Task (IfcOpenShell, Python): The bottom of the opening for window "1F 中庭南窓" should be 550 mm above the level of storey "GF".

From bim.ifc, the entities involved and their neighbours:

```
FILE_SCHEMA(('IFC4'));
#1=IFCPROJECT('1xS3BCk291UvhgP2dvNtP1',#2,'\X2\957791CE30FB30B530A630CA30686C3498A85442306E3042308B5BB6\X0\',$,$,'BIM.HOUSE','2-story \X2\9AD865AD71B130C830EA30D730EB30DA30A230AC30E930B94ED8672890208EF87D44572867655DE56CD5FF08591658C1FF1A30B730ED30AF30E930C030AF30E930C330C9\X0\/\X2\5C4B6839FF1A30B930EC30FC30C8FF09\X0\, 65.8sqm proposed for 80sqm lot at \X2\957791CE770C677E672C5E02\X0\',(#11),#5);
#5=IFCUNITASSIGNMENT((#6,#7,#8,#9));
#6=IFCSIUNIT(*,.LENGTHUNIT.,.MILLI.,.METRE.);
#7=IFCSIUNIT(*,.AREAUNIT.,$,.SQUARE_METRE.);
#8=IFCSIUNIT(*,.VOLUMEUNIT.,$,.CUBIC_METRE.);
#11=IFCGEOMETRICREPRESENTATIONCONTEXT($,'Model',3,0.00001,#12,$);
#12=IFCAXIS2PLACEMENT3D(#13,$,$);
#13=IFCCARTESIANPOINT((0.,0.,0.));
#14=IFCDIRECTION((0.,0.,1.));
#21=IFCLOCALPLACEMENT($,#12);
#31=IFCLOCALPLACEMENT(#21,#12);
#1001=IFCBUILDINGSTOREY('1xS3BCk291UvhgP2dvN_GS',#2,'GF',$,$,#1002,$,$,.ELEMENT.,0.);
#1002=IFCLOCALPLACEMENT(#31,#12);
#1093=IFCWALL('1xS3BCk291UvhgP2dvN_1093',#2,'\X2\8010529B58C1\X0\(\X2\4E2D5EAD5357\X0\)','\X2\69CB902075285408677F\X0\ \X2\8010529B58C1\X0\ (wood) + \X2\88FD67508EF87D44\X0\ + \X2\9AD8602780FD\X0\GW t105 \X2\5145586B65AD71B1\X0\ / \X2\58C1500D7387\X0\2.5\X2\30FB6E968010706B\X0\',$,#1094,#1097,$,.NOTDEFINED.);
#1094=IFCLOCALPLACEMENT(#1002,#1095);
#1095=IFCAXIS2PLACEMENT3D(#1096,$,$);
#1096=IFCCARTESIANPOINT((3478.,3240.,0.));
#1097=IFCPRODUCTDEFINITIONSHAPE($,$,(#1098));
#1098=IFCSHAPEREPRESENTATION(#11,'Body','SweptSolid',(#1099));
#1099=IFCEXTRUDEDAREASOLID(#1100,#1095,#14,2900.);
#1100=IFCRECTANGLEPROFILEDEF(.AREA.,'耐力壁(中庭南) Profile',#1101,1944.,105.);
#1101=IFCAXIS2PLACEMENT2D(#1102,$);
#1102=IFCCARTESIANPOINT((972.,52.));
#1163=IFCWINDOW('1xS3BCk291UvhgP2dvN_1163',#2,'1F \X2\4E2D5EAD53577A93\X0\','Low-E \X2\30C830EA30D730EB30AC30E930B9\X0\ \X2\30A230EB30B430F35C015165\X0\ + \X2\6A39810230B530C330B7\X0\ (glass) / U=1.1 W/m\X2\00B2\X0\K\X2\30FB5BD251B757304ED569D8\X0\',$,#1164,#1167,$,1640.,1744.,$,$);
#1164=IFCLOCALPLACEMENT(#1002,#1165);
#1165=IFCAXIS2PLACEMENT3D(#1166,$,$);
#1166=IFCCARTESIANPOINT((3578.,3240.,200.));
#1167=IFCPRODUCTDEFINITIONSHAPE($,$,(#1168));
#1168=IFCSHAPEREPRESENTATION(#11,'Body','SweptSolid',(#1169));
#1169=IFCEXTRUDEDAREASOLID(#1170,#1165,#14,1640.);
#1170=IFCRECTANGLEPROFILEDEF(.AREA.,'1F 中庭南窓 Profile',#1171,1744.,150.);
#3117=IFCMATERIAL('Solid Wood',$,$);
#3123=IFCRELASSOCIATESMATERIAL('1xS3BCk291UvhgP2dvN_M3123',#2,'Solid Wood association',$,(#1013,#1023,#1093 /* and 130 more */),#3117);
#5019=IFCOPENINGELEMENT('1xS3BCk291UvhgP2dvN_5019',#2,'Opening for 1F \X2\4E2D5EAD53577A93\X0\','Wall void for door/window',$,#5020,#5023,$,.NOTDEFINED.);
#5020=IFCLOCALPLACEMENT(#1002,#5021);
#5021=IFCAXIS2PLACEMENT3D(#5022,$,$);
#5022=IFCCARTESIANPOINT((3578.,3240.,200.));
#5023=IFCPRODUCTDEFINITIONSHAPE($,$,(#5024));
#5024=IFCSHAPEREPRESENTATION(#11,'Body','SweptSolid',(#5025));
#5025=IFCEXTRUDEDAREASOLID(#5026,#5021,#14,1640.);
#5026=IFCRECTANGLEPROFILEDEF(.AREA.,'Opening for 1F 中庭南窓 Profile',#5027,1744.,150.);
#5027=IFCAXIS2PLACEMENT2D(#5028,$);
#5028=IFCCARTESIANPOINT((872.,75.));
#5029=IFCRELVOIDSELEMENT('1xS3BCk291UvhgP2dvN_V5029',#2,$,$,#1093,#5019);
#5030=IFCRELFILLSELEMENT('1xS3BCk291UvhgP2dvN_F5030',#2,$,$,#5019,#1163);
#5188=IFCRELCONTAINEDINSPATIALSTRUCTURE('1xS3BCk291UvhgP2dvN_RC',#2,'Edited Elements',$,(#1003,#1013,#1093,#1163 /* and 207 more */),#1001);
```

```python
import numpy as np
import ifcopenshell
import ifcopenshell.api.geometry
import ifcopenshell.geom
import ifcopenshell.util.element
import ifcopenshell.util.placement
import ifcopenshell.util.shape
import ifcopenshell.util.unit

model = ifcopenshell.open("bim.ifc")
unit_scale = ifcopenshell.util.unit.calculate_unit_scale(model)

window = model.by_guid("1xS3BCk291UvhgP2dvN_1163")
opening = window.FillsVoids[0].RelatingOpeningElement
storey = ifcopenshell.util.element.get_container(window, ifc_class="IfcBuildingStorey")
level = ifcopenshell.util.placement.get_local_placement(storey.ObjectPlacement)[2, 3]

# The opening's origin need not be at the sill, so measure its lowest point.
shape = ifcopenshell.geom.create_shape(ifcopenshell.geom.settings(), opening)
bottom = ifcopenshell.util.shape.get_shape_bottom_elevation(shape, shape.geometry) / unit_scale
dz = level + 0.55 / unit_scale - bottom

shift = np.array([0.0, 0.0, dz])
# The window is not placed relative to its opening, so move both.
for product in (opening, window):
    matrix = ifcopenshell.util.placement.get_local_placement(product.ObjectPlacement)
    matrix[:3, 3] += shift
    ifcopenshell.api.geometry.edit_object_placement(model, product=product, matrix=matrix, is_si=False)

print(f"moved by {dz * unit_scale:+.3f} m")

model.write("bim-out.ifc")
```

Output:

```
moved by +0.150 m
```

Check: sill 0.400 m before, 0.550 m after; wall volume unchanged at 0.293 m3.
